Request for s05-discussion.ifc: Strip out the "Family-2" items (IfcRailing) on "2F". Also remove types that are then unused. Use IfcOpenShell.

First a look at what the model holds.

```python
import ifcopenshell
import ifcopenshell.util.element

model = ifcopenshell.open("s05-discussion.ifc")
print(model.schema)
storey = next(s for s in model.by_type("IfcBuildingStorey") if s.Name == "2F")
railings = [e for e in ifcopenshell.util.element.get_decomposition(storey) if e.is_a("IfcRailing")]
seen = {}
for e in railings:
    element_type = ifcopenshell.util.element.get_type(e)
    name = element_type.Name if element_type not in (None, e) else None
    seen[name] = seen.get(name, 0) + 1
for name, count in sorted(seen.items(), key=str):
    print(count, "x", name)
```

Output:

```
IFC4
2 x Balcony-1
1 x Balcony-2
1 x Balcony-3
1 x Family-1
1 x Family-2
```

```python
import ifcopenshell
import ifcopenshell.api.root
import ifcopenshell.util.element

model = ifcopenshell.open("s05-discussion.ifc")

storey = next(s for s in model.by_type("IfcBuildingStorey") if s.Name == "2F")
railings = [e for e in ifcopenshell.util.element.get_decomposition(storey) if e.is_a("IfcRailing")]
targets = [e for e in railings if (t := ifcopenshell.util.element.get_type(e)) not in (None, e) and t.Name == "Family-2"]
types = {ifcopenshell.util.element.get_type(e) for e in targets} - {None, *targets}

for e in targets:
    ifcopenshell.api.root.remove_product(model, product=e)
print(len(targets), "removed")

unused = [t for t in types if not ifcopenshell.util.element.get_types(t)]
for t in unused:
    ifcopenshell.api.root.remove_product(model, product=t)
print(len(unused), "unused types removed")

model.write("s05-discussion-out.ifc")
```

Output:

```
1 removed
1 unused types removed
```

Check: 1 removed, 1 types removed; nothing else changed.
